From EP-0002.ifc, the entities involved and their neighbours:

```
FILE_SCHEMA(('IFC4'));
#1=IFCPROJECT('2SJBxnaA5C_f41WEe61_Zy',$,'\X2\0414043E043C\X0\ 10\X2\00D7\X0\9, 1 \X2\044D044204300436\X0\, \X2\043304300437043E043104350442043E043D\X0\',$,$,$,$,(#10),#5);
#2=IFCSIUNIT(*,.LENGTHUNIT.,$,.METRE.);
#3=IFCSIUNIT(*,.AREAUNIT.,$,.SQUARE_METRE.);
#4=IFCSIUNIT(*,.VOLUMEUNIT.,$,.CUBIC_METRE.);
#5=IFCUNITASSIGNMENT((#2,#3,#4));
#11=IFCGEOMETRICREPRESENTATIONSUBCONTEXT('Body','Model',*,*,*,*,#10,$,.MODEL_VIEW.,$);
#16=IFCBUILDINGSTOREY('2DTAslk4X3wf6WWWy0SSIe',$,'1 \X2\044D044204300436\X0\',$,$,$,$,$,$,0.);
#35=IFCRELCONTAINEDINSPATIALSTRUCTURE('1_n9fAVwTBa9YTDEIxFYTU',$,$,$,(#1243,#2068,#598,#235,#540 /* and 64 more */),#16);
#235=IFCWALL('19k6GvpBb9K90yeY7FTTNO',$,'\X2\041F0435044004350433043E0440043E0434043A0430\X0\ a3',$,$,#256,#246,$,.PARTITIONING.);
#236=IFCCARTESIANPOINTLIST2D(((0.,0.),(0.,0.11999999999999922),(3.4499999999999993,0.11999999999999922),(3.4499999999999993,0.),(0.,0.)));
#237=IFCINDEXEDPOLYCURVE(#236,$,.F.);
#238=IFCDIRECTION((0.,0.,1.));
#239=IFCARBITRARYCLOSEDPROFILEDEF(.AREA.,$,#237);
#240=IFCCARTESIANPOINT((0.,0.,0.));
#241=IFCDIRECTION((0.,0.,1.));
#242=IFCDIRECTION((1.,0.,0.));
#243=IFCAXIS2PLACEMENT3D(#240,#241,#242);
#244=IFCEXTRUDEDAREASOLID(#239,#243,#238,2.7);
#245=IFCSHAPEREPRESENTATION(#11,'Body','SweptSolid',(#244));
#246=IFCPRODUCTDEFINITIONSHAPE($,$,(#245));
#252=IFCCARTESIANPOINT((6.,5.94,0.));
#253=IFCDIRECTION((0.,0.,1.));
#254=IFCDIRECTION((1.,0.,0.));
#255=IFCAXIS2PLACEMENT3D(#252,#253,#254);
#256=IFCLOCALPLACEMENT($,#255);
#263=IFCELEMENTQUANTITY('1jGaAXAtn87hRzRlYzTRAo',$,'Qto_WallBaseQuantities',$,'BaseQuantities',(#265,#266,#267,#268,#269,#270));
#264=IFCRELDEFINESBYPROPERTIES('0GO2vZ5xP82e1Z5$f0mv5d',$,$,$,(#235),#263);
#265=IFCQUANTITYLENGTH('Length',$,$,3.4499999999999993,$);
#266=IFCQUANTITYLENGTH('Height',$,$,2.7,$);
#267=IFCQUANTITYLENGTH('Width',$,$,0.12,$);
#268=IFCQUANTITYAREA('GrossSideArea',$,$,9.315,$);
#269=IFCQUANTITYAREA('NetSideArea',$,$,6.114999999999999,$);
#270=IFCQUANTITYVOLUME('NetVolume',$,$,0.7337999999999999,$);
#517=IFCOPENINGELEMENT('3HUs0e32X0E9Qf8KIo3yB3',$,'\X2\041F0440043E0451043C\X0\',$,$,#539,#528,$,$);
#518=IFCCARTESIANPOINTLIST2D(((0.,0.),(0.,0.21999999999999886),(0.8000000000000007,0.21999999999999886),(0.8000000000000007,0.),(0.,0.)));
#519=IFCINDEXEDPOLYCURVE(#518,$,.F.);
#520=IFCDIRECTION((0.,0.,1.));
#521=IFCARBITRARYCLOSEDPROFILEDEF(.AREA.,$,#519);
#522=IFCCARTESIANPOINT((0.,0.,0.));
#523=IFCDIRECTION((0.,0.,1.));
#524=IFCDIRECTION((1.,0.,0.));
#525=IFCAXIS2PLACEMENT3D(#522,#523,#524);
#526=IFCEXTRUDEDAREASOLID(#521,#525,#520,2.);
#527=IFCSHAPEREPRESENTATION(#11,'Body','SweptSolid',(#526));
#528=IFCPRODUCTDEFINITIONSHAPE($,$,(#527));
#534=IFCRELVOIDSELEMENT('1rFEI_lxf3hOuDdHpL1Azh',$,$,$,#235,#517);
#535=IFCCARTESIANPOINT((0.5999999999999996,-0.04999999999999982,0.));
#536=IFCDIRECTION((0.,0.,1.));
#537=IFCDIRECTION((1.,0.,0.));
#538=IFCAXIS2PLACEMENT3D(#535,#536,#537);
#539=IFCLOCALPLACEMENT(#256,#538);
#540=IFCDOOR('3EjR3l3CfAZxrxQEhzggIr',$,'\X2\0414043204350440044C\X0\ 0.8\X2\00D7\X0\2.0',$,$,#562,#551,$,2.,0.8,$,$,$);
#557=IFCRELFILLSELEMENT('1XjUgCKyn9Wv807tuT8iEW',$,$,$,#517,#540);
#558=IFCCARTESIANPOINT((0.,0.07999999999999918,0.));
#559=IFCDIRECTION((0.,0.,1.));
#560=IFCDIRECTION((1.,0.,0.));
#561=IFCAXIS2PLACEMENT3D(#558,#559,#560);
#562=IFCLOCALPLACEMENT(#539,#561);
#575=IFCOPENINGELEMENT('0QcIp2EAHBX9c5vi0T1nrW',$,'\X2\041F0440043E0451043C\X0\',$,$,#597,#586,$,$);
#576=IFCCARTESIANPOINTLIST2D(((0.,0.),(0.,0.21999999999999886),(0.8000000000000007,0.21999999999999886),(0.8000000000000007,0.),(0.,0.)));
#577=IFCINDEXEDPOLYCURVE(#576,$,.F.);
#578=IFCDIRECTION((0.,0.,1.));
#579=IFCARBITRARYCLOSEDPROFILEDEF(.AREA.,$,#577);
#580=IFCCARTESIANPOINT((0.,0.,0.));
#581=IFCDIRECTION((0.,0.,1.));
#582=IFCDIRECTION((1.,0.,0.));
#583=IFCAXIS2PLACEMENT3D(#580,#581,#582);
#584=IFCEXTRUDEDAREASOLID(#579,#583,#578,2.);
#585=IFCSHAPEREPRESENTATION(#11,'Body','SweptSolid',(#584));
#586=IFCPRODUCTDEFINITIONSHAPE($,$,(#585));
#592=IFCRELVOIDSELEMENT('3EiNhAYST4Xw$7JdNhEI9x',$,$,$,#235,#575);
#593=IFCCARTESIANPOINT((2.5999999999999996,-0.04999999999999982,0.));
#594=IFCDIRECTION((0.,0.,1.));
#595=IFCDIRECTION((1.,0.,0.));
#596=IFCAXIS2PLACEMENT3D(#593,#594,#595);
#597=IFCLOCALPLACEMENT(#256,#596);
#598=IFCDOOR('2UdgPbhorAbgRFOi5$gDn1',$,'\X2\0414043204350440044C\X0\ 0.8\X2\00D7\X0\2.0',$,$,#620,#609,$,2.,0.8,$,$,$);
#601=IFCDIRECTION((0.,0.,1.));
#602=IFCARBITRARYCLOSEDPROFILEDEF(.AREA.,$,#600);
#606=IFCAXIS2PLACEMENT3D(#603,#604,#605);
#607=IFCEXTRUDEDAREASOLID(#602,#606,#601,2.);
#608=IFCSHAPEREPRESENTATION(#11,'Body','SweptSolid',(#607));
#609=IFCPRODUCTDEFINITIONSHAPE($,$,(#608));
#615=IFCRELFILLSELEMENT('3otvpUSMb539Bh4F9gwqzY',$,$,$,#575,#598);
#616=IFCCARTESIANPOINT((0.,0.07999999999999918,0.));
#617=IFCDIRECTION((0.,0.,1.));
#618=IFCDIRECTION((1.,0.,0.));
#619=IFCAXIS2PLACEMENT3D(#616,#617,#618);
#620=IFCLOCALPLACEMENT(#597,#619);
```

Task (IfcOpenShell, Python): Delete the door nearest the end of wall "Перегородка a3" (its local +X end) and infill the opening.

```python
import ifcopenshell
import ifcopenshell.api.feature
import ifcopenshell.api.pset
import ifcopenshell.api.root
import ifcopenshell.geom
import ifcopenshell.util.element
import ifcopenshell.util.shape
import ifcopenshell.util.unit

model = ifcopenshell.open("EP-0002.ifc")
area_scale = ifcopenshell.util.unit.calculate_unit_scale(model, "AREAUNIT")
volume_scale = ifcopenshell.util.unit.calculate_unit_scale(model, "VOLUMEUNIT")
settings = ifcopenshell.geom.settings()


def volume(element):
    """Net volume in cubic metres, openings subtracted."""
    shape = ifcopenshell.geom.create_shape(settings, element)
    return ifcopenshell.util.shape.get_volume(shape.geometry)


door = model.by_guid("2UdgPbhorAbgRFOi5$gDn1")
opening = door.FillsVoids[0].RelatingOpeningElement
wall = opening.VoidsElements[0].RelatingBuildingElement
before = volume(wall)

ifcopenshell.api.root.remove_product(model, product=door)
ifcopenshell.api.feature.remove_feature(model, feature=opening)

after = volume(wall)
thickness = 0.12  # wall thickness in metres

# Update the wall's stored quantities.
qto = model.by_id(ifcopenshell.util.element.get_pset(wall, "Qto_WallBaseQuantities", should_inherit=False)["id"])
ifcopenshell.api.pset.edit_qto(model, qto=qto, properties={
    "NetSideArea": after / thickness / area_scale,
    "NetVolume": after / volume_scale,
})

print(f"wall volume {before:.3f} -> {after:.3f} m3")

model.write("EP-0002-out.ifc")
```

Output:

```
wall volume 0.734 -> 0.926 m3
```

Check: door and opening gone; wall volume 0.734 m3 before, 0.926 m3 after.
